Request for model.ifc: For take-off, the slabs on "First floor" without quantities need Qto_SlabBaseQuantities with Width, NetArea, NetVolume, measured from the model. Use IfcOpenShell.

First a look at what the model holds.

```python
import ifcopenshell
import ifcopenshell.util.element
import ifcopenshell.util.unit

model = ifcopenshell.open("model.ifc")
print(model.schema)
for unit_type in ("LENGTHUNIT", "AREAUNIT", "VOLUMEUNIT"):
    print(unit_type, ifcopenshell.util.unit.calculate_unit_scale(model, unit_type))
storey = next(s for s in model.by_type("IfcBuildingStorey") if s.Name == "First floor")
slabs = [e for e in ifcopenshell.util.element.get_decomposition(storey) if e.is_a("IfcSlab")]
for e in sorted(slabs, key=lambda e: e.id()):
    print(e.id(), e.is_a(), e.Name, list(ifcopenshell.util.element.get_psets(e, qtos_only=True)), sep=" | ")
```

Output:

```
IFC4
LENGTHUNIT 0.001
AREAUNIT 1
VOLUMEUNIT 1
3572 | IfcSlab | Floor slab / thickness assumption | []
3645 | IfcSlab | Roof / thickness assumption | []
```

```python
import ifcopenshell
import ifcopenshell.api.pset
import ifcopenshell.geom
import ifcopenshell.util.element
import ifcopenshell.util.shape
import ifcopenshell.util.unit

model = ifcopenshell.open("model.ifc")
unit_scale = ifcopenshell.util.unit.calculate_unit_scale(model)
area_scale = ifcopenshell.util.unit.calculate_unit_scale(model, "AREAUNIT")
volume_scale = ifcopenshell.util.unit.calculate_unit_scale(model, "VOLUMEUNIT")
settings = ifcopenshell.geom.settings()

storey = next(s for s in model.by_type("IfcBuildingStorey") if s.Name == "First floor")
slabs = [e for e in ifcopenshell.util.element.get_decomposition(storey) if e.is_a("IfcSlab")]

for e in sorted(slabs, key=lambda e: e.id()):
    if ifcopenshell.util.element.get_psets(e, qtos_only=True, should_inherit=False):
        continue
    # Geometry comes back in metres, in the element's own axes.
    shape = ifcopenshell.geom.create_shape(settings, e)
    values = {
        "Width": ifcopenshell.util.shape.get_z(shape.geometry) / unit_scale,
        "NetArea": ifcopenshell.util.shape.get_footprint_area(shape.geometry) / area_scale,
        "NetVolume": ifcopenshell.util.shape.get_volume(shape.geometry) / volume_scale,
    }
    qto = ifcopenshell.api.pset.add_qto(model, product=e, name="Qto_SlabBaseQuantities")
    ifcopenshell.api.pset.edit_qto(model, qto=qto, properties=values)
    print(e.id(), {k: round(v, 3) for k, v in values.items()})

model.write("model_edited.ifc")
```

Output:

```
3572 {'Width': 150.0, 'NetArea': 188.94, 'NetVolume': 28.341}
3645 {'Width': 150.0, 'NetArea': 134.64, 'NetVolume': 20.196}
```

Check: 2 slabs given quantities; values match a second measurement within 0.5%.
